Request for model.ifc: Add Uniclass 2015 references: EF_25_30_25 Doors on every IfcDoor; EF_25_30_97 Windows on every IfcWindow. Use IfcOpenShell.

First a look at what the model holds.

```python
import ifcopenshell

model = ifcopenshell.open("model.ifc")
print(model.schema)
print("classifications:", [c.Name for c in model.by_type("IfcClassification")])
for ifc_class in ("IfcDoor", "IfcRoof", "IfcStair", "IfcWall", "IfcWindow"):
    print(ifc_class, len(model.by_type(ifc_class)))
```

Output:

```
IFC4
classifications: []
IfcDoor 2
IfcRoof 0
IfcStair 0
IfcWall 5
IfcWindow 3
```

```python
import ifcopenshell
import ifcopenshell.api.classification

model = ifcopenshell.open("model.ifc")

system = ifcopenshell.api.classification.add_classification(model, classification="Uniclass 2015")

codes = {
    "IfcDoor": ("EF_25_30_25", "Doors"),
    "IfcWindow": ("EF_25_30_97", "Windows"),
}
for ifc_class, (code, name) in codes.items():
    products = model.by_type(ifc_class)
    ifcopenshell.api.classification.add_reference(
        model, products=products, classification=system, identification=code, name=name
    )
    print(code, len(products))

model.write("model-out.ifc")
```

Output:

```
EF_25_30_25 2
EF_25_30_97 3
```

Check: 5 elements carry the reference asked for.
